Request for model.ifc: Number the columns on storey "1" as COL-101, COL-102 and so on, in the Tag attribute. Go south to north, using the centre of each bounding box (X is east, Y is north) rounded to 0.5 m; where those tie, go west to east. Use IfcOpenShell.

First a look at what the model holds.

```python
import ifcopenshell
import ifcopenshell.util.element
import ifcopenshell.util.placement

model = ifcopenshell.open("model.ifc")
print(model.schema)
storey = next(s for s in model.by_type("IfcBuildingStorey") if s.Name == "1")
columns = [e for e in ifcopenshell.util.element.get_decomposition(storey) if e.is_a("IfcColumn")]
for e in sorted(columns, key=lambda e: e.id()):
    origin = ifcopenshell.util.placement.get_local_placement(e.ObjectPlacement)[:3, 3]
    print(e.id(), e.Tag, e.Name, origin.round(2) + 0.0, sep=" | ")
```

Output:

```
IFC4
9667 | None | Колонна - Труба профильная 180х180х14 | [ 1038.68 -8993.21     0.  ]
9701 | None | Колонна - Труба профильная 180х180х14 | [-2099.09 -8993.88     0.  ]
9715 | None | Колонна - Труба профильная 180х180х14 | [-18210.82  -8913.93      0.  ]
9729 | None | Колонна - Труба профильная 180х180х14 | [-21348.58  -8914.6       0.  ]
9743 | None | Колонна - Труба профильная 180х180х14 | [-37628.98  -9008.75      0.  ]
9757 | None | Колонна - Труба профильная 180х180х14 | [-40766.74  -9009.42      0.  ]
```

```python
import ifcopenshell
import ifcopenshell.geom
import ifcopenshell.util.element
import ifcopenshell.util.shape

model = ifcopenshell.open("model.ifc")
settings = ifcopenshell.geom.settings()
settings.set("use-world-coords", True)


def centre(element):
    shape = ifcopenshell.geom.create_shape(settings, element)
    return ifcopenshell.util.shape.get_bbox_centroid(shape.geometry)


storey = next(s for s in model.by_type("IfcBuildingStorey") if s.Name == "1")
columns = [e for e in ifcopenshell.util.element.get_decomposition(storey) if e.is_a("IfcColumn")]

# Insertion points can sit at a corner or the storey origin, so sort by the geometry (in metres).
centres = {e: centre(e) for e in columns}
columns.sort(key=lambda e: (round(centres[e][1] / 0.5), centres[e][0]))

for i, e in enumerate(columns, start=1):
    number = f"COL-1{i:02d}"
    e.Tag = number
    print(e.id(), number)

model.write("model-out.ifc")
```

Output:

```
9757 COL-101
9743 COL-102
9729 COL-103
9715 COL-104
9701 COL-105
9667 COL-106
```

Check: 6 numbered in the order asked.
